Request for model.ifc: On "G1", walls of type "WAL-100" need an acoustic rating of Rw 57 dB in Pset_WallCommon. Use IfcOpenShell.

First a look at what the model holds.

```python
import ifcopenshell
import ifcopenshell.util.element

model = ifcopenshell.open("model.ifc")
print(model.schema)
storey = next(s for s in model.by_type("IfcBuildingStorey") if s.Name == "G1")
walls = [e for e in ifcopenshell.util.element.get_decomposition(storey) if e.is_a("IfcWall")]
seen = {}
for e in walls:
    element_type = ifcopenshell.util.element.get_type(e)
    key = (element_type.Name if element_type != e and element_type else None, ifcopenshell.util.element.get_pset(e, "Pset_WallCommon", "AcousticRating"))
    seen[key] = seen.get(key, 0) + 1
for (name, value), count in sorted(seen.items(), key=str):
    print(count, "x", name, "|", value)
```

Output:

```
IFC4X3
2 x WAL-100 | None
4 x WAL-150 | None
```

```python
import ifcopenshell
import ifcopenshell.api.pset
import ifcopenshell.util.element

model = ifcopenshell.open("model.ifc")

storey = next(s for s in model.by_type("IfcBuildingStorey") if s.Name == "G1")
walls = [e for e in ifcopenshell.util.element.get_decomposition(storey) if e.is_a("IfcWall")]

count = 0
for e in walls:
    element_type = ifcopenshell.util.element.get_type(e)
    if element_type in (None, e) or element_type.Name != "WAL-100":
        continue
    # add_pset returns the element's existing set when there is one.
    pset = ifcopenshell.api.pset.add_pset(model, product=e, name="Pset_WallCommon")
    ifcopenshell.api.pset.edit_pset(model, pset=pset, properties={"AcousticRating": "Rw 57 dB"})
    count += 1

print(count, "walls updated")

model.write("model_v2.ifc")
```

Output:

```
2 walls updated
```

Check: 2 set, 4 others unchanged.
